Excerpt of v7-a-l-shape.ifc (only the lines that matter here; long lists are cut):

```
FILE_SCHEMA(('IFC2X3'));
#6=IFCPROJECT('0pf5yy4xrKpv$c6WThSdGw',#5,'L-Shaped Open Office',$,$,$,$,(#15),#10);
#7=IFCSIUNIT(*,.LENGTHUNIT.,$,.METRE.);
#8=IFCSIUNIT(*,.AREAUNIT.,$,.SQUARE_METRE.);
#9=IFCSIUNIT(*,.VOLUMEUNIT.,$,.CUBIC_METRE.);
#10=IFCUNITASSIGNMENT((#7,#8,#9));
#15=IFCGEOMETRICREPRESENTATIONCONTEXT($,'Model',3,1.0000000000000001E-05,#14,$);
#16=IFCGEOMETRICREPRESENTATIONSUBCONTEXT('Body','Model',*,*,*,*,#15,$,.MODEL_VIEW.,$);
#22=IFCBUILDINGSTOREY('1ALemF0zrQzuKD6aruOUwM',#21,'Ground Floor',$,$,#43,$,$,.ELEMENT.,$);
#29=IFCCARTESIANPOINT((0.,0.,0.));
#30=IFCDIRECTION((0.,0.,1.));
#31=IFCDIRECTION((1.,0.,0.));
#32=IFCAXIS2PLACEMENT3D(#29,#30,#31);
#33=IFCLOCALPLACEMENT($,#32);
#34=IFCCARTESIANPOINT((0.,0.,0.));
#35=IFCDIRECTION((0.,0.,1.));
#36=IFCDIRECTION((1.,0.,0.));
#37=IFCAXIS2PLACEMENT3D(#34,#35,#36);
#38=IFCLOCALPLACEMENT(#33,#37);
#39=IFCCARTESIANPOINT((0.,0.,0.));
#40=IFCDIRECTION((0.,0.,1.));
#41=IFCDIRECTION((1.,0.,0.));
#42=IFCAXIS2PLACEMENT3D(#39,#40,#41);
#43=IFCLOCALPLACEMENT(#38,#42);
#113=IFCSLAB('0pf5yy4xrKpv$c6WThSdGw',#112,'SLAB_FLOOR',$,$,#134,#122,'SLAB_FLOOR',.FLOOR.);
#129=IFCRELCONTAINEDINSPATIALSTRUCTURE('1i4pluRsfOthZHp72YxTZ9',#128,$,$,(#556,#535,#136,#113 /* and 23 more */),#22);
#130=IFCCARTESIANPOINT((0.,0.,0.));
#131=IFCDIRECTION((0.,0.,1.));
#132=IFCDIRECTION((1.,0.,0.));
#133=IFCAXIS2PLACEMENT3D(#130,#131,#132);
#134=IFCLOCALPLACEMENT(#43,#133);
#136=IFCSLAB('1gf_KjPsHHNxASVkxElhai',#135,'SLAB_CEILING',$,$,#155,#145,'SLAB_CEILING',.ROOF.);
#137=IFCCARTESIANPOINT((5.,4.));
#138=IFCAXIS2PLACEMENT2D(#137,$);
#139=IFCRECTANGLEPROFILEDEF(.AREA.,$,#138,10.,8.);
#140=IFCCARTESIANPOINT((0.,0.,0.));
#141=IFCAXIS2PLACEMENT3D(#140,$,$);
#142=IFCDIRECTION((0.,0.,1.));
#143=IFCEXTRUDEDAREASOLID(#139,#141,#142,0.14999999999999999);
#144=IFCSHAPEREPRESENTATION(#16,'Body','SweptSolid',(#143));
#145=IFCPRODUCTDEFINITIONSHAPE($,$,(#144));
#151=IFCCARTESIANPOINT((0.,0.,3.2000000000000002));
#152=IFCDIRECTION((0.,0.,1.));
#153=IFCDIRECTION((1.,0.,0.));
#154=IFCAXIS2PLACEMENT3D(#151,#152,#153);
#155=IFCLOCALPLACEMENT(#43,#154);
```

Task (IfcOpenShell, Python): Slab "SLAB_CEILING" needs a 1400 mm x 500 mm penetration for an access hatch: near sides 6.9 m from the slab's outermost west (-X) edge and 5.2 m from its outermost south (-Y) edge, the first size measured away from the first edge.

```python
import numpy as np
import ifcopenshell
import ifcopenshell.api.feature
import ifcopenshell.api.geometry
import ifcopenshell.api.root
import ifcopenshell.geom
import ifcopenshell.util.placement
import ifcopenshell.util.representation
import ifcopenshell.util.shape
import ifcopenshell.util.unit

model = ifcopenshell.open("v7-a-l-shape.ifc")
unit_scale = ifcopenshell.util.unit.calculate_unit_scale(model)
settings = ifcopenshell.geom.settings()


def volume(element):
    """Net volume in cubic metres, openings subtracted."""
    shape = ifcopenshell.geom.create_shape(settings, element)
    return ifcopenshell.util.shape.get_volume(shape.geometry)


slab = model.by_id(136)
before = volume(slab)

# Extent in the slab's own axes, in metres. The edges named are its -X and -Y sides.
slab_shape = ifcopenshell.geom.create_shape(settings, slab)
vertices = ifcopenshell.util.shape.get_vertices(slab_shape.geometry)
x_min, y_min, bottom = vertices.min(axis=0)
top = vertices[:, 2].max()

opening = ifcopenshell.api.root.create_entity(model, ifc_class="IfcOpeningElement", name="Access hatch opening")
context = ifcopenshell.util.representation.get_context(model, "Model", "Body", "MODEL_VIEW")
width, depth = 1.4, 0.5
outline = [(0.0, 0.0), (width, 0.0), (width, depth), (0.0, depth), (0.0, 0.0)]
# Overshoot both faces by 50 mm so the cut is clean.
shape = ifcopenshell.api.geometry.add_slab_representation(
    model, context=context, depth=top - bottom + 0.1, polyline=outline
)
ifcopenshell.api.geometry.assign_representation(model, product=opening, representation=shape)

matrix = ifcopenshell.util.placement.get_local_placement(slab.ObjectPlacement)
matrix[:, 3] = matrix @ np.append(np.array([x_min + 6.9, y_min + 5.2, bottom - 0.05]) / unit_scale, 1.0)
ifcopenshell.api.geometry.edit_object_placement(model, product=opening, matrix=matrix, is_si=False)
ifcopenshell.api.feature.add_feature(model, feature=opening, element=slab)

after = volume(slab)

print(f"slab volume {before:.3f} -> {after:.3f} m3")

model.write("v7-a-l-shape_v2.ifc")
```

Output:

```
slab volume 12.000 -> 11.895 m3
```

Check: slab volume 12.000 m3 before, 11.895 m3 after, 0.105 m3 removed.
